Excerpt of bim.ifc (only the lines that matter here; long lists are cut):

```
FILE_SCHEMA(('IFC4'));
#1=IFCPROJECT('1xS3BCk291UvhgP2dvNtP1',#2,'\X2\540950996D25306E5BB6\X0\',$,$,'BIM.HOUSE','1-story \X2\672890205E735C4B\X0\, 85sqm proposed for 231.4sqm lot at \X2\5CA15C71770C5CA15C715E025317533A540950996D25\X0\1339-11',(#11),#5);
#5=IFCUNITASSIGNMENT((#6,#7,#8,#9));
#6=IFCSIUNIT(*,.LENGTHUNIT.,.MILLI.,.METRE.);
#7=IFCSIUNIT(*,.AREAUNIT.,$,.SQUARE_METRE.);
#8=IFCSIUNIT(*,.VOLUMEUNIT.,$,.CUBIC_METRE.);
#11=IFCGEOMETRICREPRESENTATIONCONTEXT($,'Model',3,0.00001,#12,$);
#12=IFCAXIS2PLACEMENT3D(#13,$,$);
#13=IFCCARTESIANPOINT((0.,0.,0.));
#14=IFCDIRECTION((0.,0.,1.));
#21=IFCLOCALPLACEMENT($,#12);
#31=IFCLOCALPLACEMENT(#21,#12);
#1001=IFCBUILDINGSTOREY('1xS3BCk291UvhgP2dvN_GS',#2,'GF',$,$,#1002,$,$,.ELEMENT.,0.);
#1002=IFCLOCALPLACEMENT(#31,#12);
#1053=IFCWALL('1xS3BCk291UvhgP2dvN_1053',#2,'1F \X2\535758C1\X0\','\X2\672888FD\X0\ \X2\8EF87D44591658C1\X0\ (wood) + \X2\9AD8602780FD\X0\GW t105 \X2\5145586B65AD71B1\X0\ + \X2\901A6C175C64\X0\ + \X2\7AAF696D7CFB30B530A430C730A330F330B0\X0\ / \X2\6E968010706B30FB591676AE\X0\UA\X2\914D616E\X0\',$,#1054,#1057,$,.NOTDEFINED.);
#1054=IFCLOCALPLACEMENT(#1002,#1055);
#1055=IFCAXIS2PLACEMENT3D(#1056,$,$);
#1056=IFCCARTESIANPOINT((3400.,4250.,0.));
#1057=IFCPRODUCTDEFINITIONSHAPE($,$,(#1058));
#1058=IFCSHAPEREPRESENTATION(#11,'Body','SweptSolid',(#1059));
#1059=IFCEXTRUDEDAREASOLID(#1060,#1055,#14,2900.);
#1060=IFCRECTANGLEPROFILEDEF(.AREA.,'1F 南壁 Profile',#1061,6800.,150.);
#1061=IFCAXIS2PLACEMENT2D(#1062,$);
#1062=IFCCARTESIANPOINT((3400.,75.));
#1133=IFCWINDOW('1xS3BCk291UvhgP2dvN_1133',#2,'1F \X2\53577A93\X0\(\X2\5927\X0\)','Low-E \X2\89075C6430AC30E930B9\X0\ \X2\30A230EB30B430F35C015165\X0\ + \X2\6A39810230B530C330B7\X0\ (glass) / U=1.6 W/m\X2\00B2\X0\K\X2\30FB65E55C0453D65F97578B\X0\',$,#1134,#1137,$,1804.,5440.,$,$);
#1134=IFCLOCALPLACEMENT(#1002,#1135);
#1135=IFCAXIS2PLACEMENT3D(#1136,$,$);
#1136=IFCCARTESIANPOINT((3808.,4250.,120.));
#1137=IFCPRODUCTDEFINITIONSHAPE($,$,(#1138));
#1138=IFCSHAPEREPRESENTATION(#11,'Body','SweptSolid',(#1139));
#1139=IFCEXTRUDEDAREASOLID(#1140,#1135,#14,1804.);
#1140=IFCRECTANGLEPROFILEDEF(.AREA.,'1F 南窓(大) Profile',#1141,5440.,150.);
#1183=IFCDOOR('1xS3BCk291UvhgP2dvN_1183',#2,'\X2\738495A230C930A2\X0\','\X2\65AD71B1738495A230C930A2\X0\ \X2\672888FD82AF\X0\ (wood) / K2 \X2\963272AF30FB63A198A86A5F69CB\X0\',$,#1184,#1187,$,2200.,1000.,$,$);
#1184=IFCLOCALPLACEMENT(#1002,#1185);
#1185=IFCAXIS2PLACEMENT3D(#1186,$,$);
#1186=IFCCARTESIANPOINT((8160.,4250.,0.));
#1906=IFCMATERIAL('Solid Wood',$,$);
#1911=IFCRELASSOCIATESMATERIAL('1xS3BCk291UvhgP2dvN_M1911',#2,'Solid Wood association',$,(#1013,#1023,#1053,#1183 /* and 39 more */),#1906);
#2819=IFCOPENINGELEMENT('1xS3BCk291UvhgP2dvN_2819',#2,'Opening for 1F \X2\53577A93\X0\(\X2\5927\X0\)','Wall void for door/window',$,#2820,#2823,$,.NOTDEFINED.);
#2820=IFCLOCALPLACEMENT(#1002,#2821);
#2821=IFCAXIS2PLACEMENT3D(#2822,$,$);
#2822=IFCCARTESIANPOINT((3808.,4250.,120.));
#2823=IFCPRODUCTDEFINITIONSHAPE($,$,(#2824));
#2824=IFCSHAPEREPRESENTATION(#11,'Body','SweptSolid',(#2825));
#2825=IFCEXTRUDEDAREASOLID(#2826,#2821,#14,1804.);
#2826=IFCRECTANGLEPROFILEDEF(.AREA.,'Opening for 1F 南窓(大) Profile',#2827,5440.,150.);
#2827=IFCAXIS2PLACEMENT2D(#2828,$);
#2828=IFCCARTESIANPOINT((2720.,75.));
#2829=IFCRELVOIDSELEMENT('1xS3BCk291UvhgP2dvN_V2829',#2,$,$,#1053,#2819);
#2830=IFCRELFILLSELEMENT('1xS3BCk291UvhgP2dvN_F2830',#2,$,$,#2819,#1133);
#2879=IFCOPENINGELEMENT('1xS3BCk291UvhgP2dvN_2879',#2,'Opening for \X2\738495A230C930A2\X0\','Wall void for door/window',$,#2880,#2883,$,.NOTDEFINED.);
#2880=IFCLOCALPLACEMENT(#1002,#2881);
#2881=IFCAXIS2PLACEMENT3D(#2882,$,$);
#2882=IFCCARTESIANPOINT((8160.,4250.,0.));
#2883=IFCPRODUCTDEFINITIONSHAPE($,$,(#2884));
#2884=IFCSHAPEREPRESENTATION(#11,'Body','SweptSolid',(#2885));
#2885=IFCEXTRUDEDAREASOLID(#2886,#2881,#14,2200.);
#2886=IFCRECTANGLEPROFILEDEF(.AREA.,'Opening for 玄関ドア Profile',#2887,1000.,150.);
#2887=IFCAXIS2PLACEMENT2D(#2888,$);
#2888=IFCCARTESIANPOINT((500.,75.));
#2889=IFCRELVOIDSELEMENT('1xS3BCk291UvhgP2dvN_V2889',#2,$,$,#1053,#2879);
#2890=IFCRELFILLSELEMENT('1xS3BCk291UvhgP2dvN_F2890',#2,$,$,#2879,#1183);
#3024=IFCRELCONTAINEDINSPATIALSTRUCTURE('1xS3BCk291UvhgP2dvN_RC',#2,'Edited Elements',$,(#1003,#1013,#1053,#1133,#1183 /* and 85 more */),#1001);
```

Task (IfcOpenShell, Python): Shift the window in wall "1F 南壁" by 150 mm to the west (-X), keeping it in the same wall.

```python
import ifcopenshell
import ifcopenshell.api.geometry
import ifcopenshell.util.placement
import ifcopenshell.util.unit

model = ifcopenshell.open("bim.ifc")
unit_scale = ifcopenshell.util.unit.calculate_unit_scale(model)

window = model.by_guid("1xS3BCk291UvhgP2dvN_1133")
opening = window.FillsVoids[0].RelatingOpeningElement
wall = opening.VoidsElements[0].RelatingBuildingElement

wall_matrix = ifcopenshell.util.placement.get_local_placement(wall.ObjectPlacement)
shift = wall_matrix[:3, 0] * -0.15 / unit_scale
before = ifcopenshell.util.placement.get_local_placement(window.ObjectPlacement)[:3, 3].copy()

# The window is not placed relative to its opening, so move both.
for product in (opening, window):
    matrix = ifcopenshell.util.placement.get_local_placement(product.ObjectPlacement)
    matrix[:3, 3] += shift
    ifcopenshell.api.geometry.edit_object_placement(model, product=product, matrix=matrix, is_si=False)

after = ifcopenshell.util.placement.get_local_placement(window.ObjectPlacement)[:3, 3]
print("window moved by", (after - before).round(3) + 0.0)

model.write("bim_rev.ifc")
```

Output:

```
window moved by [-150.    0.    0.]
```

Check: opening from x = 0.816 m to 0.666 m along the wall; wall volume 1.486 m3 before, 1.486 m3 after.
